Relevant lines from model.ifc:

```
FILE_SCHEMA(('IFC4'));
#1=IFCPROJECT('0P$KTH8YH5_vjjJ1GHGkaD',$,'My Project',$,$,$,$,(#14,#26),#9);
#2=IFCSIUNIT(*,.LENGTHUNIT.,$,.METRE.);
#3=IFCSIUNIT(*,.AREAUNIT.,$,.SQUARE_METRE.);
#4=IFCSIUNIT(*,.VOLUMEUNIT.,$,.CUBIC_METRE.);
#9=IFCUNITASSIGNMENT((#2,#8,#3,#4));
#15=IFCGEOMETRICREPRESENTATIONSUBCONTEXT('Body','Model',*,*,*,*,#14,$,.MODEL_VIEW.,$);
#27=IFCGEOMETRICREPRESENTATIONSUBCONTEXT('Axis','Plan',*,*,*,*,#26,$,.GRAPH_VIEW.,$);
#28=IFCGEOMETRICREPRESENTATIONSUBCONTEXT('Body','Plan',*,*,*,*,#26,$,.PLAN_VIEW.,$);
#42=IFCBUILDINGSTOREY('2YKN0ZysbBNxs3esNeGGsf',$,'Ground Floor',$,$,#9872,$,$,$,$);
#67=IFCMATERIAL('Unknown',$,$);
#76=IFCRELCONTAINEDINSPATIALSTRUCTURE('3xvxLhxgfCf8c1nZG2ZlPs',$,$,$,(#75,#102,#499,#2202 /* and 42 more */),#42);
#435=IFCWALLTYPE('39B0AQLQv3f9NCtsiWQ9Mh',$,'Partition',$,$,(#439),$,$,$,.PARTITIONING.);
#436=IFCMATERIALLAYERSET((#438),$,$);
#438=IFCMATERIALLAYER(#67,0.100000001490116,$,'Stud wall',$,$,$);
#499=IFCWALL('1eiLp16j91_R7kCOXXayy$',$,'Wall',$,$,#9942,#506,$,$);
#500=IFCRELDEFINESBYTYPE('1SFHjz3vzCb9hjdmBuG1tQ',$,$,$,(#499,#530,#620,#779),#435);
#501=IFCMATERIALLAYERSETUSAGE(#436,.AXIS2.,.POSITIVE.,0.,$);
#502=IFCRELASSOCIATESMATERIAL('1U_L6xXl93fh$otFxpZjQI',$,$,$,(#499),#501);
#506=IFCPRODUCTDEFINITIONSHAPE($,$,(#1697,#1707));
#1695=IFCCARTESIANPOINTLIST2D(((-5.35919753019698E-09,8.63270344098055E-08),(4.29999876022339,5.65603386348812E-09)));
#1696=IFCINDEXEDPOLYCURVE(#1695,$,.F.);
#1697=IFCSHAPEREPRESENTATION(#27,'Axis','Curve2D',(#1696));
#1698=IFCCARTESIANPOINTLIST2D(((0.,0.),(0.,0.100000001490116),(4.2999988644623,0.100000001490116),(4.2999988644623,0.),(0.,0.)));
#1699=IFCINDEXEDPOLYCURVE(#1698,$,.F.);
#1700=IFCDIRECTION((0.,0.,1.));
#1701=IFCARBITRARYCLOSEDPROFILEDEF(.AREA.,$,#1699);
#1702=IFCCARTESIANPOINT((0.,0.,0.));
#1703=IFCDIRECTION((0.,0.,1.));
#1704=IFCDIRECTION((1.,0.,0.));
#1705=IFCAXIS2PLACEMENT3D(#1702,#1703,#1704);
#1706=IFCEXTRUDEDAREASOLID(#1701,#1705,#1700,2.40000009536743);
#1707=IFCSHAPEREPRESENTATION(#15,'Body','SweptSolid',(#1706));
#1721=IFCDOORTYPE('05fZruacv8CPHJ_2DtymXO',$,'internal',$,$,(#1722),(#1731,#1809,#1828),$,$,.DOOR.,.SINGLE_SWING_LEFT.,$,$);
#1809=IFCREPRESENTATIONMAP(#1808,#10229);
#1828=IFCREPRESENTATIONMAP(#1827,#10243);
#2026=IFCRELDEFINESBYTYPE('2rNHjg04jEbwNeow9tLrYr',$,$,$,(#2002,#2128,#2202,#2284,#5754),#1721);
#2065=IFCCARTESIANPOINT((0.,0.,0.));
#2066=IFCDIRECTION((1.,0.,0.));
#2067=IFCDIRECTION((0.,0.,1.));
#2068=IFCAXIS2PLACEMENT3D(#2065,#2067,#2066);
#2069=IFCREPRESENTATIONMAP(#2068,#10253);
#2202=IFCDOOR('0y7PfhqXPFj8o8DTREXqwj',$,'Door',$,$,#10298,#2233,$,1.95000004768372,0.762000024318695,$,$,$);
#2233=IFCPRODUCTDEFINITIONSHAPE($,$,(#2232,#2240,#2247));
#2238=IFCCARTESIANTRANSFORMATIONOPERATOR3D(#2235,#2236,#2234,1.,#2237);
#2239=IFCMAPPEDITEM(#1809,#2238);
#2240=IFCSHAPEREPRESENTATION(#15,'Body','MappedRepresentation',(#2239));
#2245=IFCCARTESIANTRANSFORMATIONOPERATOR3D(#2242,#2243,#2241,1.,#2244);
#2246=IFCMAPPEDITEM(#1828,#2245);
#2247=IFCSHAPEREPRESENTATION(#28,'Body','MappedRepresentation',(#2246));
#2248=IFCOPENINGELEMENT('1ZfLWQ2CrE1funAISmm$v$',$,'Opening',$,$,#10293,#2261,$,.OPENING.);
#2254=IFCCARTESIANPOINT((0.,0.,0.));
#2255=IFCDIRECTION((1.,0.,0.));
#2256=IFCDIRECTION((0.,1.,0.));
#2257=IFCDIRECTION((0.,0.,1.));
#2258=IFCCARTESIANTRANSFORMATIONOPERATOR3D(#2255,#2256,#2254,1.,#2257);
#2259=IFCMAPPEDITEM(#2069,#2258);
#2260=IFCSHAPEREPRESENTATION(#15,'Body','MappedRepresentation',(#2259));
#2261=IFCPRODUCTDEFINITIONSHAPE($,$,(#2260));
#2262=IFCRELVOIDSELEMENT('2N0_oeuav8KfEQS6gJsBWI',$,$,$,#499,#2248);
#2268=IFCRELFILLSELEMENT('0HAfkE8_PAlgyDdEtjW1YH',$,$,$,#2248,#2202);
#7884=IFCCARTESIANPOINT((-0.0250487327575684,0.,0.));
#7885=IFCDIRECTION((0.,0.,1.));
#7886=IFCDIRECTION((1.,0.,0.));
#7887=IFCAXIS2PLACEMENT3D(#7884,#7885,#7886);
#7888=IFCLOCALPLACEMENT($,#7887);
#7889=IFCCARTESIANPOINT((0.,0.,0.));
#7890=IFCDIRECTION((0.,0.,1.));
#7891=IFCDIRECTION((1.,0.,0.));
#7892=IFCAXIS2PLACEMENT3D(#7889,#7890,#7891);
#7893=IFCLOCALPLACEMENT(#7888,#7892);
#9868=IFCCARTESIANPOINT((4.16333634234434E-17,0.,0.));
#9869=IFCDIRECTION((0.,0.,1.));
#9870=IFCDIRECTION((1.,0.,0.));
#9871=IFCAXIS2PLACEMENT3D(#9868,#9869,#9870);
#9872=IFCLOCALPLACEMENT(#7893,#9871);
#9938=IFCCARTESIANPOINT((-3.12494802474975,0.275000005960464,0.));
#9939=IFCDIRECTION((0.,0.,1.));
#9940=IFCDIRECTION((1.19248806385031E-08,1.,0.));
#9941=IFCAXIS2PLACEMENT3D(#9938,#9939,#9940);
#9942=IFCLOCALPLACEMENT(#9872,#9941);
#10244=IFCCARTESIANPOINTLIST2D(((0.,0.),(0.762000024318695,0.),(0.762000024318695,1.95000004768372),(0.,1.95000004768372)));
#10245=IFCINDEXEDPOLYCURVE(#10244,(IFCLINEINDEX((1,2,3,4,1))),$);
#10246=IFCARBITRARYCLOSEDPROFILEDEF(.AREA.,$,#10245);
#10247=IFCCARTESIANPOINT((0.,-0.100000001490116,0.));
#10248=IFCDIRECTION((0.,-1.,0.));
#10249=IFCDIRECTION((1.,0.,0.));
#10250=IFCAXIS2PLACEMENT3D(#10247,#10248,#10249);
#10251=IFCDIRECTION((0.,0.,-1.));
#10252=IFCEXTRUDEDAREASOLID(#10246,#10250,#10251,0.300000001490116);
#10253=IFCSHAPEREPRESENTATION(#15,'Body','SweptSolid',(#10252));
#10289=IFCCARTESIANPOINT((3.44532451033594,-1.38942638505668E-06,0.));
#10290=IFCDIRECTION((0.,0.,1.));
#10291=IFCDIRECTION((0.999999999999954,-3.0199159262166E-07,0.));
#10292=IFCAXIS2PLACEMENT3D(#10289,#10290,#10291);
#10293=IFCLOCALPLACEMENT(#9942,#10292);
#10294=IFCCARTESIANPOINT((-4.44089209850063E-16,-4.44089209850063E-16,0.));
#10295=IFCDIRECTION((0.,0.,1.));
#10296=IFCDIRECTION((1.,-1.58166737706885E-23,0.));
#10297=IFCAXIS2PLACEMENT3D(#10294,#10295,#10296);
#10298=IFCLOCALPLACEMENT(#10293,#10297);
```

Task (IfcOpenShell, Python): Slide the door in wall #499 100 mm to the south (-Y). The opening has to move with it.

```python
import ifcopenshell
import ifcopenshell.api.geometry
import ifcopenshell.util.placement
import ifcopenshell.util.unit

model = ifcopenshell.open("model.ifc")
unit_scale = ifcopenshell.util.unit.calculate_unit_scale(model)

door = model.by_guid("0y7PfhqXPFj8o8DTREXqwj")
opening = door.FillsVoids[0].RelatingOpeningElement
wall = opening.VoidsElements[0].RelatingBuildingElement

wall_matrix = ifcopenshell.util.placement.get_local_placement(wall.ObjectPlacement)
shift = wall_matrix[:3, 0] * -0.1 / unit_scale
before = ifcopenshell.util.placement.get_local_placement(door.ObjectPlacement)[:3, 3].copy()

# The door is placed relative to its opening, so it follows when the opening moves.
matrix = ifcopenshell.util.placement.get_local_placement(opening.ObjectPlacement)
matrix[:3, 3] += shift
ifcopenshell.api.geometry.edit_object_placement(
    model, product=opening, matrix=matrix, is_si=False, should_transform_children=True
)

after = ifcopenshell.util.placement.get_local_placement(door.ObjectPlacement)[:3, 3]
print("door moved by", (after - before).round(3) + 0.0)

model.write("model-out.ifc")
```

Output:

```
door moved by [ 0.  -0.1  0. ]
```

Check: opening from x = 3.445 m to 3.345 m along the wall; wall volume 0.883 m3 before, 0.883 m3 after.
